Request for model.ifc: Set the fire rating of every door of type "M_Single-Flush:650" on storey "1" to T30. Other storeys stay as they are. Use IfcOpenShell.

First a look at what the model holds.

```python
import ifcopenshell
import ifcopenshell.util.element

model = ifcopenshell.open("model.ifc")
print(model.schema)
storey = next(s for s in model.by_type("IfcBuildingStorey") if s.Name == "1")
doors = [e for e in ifcopenshell.util.element.get_decomposition(storey) if e.is_a("IfcDoor")]
seen = {}
for e in doors:
    element_type = ifcopenshell.util.element.get_type(e)
    key = (element_type.Name if element_type != e and element_type else None, ifcopenshell.util.element.get_pset(e, "Pset_DoorCommon", "FireRating"))
    seen[key] = seen.get(key, 0) + 1
for (name, value), count in sorted(seen.items(), key=str):
    print(count, "x", name, "|", value)
```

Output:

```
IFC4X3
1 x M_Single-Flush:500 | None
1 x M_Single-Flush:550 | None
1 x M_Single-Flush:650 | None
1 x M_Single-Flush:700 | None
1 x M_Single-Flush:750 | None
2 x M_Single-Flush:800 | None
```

```python
import ifcopenshell
import ifcopenshell.api.pset
import ifcopenshell.util.element

model = ifcopenshell.open("model.ifc")

storey = next(s for s in model.by_type("IfcBuildingStorey") if s.Name == "1")
doors = [e for e in ifcopenshell.util.element.get_decomposition(storey) if e.is_a("IfcDoor")]

count = 0
for e in doors:
    element_type = ifcopenshell.util.element.get_type(e)
    if element_type in (None, e) or element_type.Name != "M_Single-Flush:650":
        continue
    # add_pset returns the element's existing set when there is one.
    pset = ifcopenshell.api.pset.add_pset(model, product=e, name="Pset_DoorCommon")
    ifcopenshell.api.pset.edit_pset(model, pset=pset, properties={"FireRating": "T30"})
    count += 1

print(count, "doors updated")

model.write("model_updated.ifc")
```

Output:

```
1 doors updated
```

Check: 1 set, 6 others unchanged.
